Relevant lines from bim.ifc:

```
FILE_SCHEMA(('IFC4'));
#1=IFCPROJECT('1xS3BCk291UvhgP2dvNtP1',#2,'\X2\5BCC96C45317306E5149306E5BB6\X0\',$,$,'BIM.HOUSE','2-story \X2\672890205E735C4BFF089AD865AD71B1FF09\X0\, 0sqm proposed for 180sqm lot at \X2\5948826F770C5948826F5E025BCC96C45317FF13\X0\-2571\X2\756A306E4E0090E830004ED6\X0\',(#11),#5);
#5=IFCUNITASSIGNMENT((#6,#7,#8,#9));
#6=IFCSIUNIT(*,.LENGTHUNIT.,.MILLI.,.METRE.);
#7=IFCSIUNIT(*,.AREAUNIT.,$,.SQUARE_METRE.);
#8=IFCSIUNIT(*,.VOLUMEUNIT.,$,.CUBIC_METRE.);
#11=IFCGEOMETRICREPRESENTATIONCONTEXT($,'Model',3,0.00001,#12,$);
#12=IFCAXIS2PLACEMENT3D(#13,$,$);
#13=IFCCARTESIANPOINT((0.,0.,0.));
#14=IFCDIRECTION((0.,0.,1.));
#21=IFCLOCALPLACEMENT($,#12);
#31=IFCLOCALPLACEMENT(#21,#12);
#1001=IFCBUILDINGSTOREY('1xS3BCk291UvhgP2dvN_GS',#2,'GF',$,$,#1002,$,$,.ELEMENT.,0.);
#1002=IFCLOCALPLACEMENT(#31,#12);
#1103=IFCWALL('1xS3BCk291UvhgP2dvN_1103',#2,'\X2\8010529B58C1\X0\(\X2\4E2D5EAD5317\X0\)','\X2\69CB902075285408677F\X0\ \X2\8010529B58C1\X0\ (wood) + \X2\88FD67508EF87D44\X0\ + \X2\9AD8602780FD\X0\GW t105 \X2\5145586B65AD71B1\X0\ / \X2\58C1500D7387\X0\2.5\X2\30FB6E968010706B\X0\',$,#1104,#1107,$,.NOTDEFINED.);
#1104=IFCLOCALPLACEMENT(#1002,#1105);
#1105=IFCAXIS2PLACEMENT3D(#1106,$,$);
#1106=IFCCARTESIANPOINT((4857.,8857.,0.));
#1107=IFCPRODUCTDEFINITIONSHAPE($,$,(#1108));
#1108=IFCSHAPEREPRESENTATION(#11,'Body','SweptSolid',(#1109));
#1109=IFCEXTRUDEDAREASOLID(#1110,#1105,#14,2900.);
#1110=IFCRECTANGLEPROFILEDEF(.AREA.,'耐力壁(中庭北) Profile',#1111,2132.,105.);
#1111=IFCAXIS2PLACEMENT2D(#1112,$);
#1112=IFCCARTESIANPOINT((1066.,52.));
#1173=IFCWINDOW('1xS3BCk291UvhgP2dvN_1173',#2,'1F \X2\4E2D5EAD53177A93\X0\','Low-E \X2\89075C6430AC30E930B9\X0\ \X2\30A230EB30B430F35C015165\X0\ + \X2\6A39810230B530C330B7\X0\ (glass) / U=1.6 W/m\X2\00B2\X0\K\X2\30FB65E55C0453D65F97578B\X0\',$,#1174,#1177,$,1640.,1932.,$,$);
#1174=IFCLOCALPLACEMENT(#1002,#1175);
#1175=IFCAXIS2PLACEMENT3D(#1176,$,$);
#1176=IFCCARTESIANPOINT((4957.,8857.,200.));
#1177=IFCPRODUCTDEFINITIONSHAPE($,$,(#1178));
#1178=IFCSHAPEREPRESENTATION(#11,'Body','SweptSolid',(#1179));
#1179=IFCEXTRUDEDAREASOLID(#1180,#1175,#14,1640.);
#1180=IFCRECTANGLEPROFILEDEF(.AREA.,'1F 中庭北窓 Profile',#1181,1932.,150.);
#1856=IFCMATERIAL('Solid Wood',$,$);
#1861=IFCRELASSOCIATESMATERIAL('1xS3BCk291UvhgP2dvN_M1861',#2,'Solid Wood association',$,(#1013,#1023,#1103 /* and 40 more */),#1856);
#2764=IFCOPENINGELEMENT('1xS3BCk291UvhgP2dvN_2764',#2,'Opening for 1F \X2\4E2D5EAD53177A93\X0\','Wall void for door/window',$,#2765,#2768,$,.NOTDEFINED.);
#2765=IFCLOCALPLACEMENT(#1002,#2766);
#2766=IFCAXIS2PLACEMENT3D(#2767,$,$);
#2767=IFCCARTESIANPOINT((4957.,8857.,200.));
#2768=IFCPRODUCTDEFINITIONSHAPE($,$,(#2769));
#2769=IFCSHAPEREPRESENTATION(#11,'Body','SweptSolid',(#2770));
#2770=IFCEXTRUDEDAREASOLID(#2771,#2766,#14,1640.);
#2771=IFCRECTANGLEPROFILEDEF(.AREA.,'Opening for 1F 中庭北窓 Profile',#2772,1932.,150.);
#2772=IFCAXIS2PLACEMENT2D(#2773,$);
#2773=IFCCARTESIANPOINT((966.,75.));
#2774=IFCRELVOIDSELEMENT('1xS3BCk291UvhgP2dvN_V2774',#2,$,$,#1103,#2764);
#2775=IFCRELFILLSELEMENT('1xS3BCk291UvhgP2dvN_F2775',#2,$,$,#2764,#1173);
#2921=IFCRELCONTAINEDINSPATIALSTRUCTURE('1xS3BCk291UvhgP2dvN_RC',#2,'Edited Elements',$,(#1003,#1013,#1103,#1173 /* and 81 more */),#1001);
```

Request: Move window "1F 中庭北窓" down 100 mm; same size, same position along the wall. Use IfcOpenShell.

```python
import numpy as np
import ifcopenshell
import ifcopenshell.api.geometry
import ifcopenshell.util.placement
import ifcopenshell.util.unit

model = ifcopenshell.open("bim.ifc")
unit_scale = ifcopenshell.util.unit.calculate_unit_scale(model)

window = model.by_guid("1xS3BCk291UvhgP2dvN_1173")
opening = window.FillsVoids[0].RelatingOpeningElement
dz = -0.1 / unit_scale

shift = np.array([0.0, 0.0, dz])
# The window is not placed relative to its opening, so move both.
for product in (opening, window):
    matrix = ifcopenshell.util.placement.get_local_placement(product.ObjectPlacement)
    matrix[:3, 3] += shift
    ifcopenshell.api.geometry.edit_object_placement(model, product=product, matrix=matrix, is_si=False)

print(f"moved by {dz * unit_scale:+.3f} m")

model.write("bim_rev.ifc")
```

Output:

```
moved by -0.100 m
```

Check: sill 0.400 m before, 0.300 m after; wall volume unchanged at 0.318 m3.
